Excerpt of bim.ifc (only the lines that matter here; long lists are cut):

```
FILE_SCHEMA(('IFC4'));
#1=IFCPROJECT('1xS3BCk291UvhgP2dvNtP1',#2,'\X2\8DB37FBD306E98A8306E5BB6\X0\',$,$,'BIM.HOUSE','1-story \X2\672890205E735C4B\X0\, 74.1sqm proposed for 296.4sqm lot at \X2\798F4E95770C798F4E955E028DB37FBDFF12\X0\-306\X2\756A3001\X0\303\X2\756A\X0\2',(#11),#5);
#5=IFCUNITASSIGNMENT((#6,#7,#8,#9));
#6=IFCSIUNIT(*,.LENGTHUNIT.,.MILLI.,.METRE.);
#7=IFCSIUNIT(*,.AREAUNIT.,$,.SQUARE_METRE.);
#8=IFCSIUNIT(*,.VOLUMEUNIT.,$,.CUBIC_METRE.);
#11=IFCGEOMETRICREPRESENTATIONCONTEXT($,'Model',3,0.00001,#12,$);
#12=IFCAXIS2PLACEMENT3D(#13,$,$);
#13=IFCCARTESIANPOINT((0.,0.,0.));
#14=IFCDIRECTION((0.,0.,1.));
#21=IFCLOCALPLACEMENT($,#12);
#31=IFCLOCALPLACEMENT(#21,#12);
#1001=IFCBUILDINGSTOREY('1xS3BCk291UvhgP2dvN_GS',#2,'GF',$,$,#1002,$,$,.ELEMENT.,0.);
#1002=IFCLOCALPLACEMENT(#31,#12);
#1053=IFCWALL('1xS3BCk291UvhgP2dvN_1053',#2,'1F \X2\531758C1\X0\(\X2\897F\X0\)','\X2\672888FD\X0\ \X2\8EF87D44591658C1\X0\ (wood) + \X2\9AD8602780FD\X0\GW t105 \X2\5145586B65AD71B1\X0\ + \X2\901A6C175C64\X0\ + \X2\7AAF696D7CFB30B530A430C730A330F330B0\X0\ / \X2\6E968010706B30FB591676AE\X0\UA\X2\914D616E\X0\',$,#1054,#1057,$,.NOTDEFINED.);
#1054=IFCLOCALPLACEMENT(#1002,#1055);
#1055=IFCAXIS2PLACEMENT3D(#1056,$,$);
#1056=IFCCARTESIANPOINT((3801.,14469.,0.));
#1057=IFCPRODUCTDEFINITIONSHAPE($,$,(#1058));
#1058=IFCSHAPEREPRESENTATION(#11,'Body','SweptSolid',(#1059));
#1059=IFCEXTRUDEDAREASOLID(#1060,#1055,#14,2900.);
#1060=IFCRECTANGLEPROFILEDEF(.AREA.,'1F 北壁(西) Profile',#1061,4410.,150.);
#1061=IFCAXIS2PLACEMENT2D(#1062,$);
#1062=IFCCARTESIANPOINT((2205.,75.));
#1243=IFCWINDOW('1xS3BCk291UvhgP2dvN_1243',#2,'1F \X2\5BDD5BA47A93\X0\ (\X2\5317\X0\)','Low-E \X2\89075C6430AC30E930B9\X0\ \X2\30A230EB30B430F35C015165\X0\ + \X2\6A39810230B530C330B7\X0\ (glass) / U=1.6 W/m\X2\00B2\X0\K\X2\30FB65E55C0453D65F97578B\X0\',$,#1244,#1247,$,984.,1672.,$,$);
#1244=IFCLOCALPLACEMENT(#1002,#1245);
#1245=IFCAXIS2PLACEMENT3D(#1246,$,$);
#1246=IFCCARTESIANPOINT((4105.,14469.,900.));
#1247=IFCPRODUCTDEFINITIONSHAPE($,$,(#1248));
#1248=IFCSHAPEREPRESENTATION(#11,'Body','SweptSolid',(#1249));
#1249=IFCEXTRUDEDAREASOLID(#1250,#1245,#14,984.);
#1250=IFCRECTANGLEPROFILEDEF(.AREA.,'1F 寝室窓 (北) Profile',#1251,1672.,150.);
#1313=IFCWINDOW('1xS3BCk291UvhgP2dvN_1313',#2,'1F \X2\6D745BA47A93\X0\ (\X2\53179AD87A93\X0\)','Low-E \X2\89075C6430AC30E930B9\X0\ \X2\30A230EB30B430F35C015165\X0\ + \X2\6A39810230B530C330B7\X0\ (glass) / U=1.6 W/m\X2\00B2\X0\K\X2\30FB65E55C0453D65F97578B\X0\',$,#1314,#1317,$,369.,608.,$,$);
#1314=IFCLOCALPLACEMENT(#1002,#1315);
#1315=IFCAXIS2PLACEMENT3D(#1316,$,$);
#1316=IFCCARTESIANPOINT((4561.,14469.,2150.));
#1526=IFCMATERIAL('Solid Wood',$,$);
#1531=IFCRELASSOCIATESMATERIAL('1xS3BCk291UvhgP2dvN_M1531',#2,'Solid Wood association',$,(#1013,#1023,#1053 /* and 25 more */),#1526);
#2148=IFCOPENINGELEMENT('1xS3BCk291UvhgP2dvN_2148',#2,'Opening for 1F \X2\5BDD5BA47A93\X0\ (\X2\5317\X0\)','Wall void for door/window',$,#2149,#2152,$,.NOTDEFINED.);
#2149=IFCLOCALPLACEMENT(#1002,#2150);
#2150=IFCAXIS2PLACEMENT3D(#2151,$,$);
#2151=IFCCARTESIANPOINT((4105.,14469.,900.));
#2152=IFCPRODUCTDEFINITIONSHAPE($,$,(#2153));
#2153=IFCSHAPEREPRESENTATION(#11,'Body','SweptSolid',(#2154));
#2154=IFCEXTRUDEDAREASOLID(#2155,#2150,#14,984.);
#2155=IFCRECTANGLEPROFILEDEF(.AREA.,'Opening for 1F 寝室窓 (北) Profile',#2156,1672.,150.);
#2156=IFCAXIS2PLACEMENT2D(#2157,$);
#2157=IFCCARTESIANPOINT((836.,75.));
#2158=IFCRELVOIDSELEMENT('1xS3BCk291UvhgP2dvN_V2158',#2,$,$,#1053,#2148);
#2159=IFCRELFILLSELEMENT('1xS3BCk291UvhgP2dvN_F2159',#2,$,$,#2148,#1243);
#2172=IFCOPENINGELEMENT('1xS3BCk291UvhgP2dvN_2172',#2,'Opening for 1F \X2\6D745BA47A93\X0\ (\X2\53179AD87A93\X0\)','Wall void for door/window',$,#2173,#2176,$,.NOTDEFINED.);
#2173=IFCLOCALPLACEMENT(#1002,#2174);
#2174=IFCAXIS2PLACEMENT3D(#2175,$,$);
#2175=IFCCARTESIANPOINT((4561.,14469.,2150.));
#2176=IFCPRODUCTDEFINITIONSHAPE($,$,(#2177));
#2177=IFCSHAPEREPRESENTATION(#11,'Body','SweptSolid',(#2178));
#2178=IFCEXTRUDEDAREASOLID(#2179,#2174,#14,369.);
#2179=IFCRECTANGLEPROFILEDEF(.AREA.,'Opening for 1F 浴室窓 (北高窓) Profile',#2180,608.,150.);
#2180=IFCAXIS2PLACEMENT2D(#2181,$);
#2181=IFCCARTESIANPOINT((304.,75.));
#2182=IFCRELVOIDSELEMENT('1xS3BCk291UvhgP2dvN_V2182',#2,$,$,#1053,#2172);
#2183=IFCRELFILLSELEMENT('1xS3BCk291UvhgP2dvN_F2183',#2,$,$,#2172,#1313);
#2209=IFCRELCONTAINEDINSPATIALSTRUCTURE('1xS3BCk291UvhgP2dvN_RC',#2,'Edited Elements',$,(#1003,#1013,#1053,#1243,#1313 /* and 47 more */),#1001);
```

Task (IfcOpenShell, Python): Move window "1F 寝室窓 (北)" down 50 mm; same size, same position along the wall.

```python
import numpy as np
import ifcopenshell
import ifcopenshell.api.geometry
import ifcopenshell.util.placement
import ifcopenshell.util.unit

model = ifcopenshell.open("bim.ifc")
unit_scale = ifcopenshell.util.unit.calculate_unit_scale(model)

window = model.by_id(1243)
opening = window.FillsVoids[0].RelatingOpeningElement
dz = -0.05 / unit_scale

shift = np.array([0.0, 0.0, dz])
# The window is not placed relative to its opening, so move both.
for product in (opening, window):
    matrix = ifcopenshell.util.placement.get_local_placement(product.ObjectPlacement)
    matrix[:3, 3] += shift
    ifcopenshell.api.geometry.edit_object_placement(model, product=product, matrix=matrix, is_si=False)

print(f"moved by {dz * unit_scale:+.3f} m")

model.write("bim_updated.ifc")
```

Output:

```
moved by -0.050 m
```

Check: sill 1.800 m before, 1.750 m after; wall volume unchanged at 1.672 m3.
